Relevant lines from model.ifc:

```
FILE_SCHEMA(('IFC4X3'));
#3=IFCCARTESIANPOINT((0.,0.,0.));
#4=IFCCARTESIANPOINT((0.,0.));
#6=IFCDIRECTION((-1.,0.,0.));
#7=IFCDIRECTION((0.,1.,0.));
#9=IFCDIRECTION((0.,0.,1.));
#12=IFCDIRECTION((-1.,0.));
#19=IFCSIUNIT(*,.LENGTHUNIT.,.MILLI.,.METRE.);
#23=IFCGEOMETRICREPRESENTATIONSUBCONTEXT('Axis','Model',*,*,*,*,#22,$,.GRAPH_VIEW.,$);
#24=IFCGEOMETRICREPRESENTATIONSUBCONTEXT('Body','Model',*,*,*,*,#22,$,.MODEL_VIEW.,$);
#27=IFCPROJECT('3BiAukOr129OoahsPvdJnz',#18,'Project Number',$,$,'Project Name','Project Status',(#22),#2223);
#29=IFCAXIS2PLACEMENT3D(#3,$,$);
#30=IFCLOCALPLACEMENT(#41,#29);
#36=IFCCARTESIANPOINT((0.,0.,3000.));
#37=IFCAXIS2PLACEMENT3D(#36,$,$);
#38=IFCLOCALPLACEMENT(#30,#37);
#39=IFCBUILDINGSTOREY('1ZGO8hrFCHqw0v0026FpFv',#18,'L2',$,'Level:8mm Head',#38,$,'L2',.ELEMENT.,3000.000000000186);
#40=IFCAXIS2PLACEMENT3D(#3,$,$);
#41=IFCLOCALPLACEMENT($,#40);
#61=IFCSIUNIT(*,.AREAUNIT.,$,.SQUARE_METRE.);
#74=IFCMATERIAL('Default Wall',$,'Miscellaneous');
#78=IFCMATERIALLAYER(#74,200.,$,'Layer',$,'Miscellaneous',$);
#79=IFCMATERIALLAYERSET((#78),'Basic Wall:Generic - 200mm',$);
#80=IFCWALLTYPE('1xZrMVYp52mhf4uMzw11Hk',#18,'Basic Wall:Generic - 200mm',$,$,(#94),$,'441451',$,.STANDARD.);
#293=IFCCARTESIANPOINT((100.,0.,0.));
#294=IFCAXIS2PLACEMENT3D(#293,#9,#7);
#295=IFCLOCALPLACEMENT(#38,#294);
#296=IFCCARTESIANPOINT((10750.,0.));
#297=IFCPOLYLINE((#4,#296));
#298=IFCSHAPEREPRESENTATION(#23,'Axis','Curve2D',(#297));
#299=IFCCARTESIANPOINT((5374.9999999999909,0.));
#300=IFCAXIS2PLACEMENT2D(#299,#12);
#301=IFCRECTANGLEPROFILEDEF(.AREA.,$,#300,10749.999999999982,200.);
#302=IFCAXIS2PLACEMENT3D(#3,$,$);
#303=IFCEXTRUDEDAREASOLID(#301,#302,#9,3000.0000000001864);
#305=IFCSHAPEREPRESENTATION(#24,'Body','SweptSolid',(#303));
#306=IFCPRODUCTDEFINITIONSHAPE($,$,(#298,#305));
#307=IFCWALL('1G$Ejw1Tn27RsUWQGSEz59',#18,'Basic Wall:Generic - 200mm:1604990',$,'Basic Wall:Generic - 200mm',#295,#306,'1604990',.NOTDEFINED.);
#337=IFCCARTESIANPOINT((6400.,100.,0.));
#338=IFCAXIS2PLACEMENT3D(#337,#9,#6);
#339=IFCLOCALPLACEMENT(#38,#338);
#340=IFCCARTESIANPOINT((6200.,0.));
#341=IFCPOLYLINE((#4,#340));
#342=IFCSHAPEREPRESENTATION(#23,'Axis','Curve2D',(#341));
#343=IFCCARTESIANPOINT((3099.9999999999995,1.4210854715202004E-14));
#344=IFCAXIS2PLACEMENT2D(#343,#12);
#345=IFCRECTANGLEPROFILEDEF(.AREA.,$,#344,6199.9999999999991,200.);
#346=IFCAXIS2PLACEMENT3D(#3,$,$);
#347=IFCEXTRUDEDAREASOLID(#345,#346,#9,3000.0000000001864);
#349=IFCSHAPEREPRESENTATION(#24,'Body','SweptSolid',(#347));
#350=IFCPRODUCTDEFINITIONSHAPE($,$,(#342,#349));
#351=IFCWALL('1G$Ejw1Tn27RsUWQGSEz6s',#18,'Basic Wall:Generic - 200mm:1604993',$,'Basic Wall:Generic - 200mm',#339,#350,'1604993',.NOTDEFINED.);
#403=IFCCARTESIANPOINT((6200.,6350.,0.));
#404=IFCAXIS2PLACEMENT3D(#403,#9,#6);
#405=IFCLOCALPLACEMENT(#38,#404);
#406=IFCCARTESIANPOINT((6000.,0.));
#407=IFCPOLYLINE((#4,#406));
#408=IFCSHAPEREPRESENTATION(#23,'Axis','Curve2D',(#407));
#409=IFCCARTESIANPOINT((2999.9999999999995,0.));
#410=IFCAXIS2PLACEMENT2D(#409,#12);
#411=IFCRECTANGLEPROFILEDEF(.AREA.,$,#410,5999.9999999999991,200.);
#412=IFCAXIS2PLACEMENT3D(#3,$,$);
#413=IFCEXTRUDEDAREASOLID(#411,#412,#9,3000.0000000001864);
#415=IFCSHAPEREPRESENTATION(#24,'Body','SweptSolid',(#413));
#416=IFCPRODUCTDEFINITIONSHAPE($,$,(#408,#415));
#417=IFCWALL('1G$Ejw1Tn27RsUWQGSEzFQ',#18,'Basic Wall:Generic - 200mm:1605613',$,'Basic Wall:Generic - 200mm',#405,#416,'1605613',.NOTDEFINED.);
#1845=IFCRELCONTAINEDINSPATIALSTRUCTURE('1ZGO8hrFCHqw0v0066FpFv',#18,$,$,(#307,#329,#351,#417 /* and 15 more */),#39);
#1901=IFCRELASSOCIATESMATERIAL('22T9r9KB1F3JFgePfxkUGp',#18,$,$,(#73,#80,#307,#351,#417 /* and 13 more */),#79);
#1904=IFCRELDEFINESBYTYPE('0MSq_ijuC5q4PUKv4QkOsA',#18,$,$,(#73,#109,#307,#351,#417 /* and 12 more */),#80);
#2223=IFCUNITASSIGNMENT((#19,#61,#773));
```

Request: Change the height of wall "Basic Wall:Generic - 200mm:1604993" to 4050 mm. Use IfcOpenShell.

```python
import ifcopenshell
import ifcopenshell.geom
import ifcopenshell.util.representation
import ifcopenshell.util.shape
import ifcopenshell.util.unit

model = ifcopenshell.open("model.ifc")
unit_scale = ifcopenshell.util.unit.calculate_unit_scale(model)
settings = ifcopenshell.geom.settings()


def volume(element):
    """Net volume in cubic metres, openings subtracted."""
    shape = ifcopenshell.geom.create_shape(settings, element)
    return ifcopenshell.util.shape.get_volume(shape.geometry)


wall = model.by_id(351)
before = volume(wall)

body = ifcopenshell.util.representation.get_representation(wall, "Model", "Body")
solid = body.Items[0]
old_height = solid.Depth
solid.Depth = 4.05 / unit_scale
after = volume(wall)

print(f"height {old_height:g} -> {solid.Depth:g}, volume {before:.3f} -> {after:.3f} m3")

model.write("model_updated.ifc")
```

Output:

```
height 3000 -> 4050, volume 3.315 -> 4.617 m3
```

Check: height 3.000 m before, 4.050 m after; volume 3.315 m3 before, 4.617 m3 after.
